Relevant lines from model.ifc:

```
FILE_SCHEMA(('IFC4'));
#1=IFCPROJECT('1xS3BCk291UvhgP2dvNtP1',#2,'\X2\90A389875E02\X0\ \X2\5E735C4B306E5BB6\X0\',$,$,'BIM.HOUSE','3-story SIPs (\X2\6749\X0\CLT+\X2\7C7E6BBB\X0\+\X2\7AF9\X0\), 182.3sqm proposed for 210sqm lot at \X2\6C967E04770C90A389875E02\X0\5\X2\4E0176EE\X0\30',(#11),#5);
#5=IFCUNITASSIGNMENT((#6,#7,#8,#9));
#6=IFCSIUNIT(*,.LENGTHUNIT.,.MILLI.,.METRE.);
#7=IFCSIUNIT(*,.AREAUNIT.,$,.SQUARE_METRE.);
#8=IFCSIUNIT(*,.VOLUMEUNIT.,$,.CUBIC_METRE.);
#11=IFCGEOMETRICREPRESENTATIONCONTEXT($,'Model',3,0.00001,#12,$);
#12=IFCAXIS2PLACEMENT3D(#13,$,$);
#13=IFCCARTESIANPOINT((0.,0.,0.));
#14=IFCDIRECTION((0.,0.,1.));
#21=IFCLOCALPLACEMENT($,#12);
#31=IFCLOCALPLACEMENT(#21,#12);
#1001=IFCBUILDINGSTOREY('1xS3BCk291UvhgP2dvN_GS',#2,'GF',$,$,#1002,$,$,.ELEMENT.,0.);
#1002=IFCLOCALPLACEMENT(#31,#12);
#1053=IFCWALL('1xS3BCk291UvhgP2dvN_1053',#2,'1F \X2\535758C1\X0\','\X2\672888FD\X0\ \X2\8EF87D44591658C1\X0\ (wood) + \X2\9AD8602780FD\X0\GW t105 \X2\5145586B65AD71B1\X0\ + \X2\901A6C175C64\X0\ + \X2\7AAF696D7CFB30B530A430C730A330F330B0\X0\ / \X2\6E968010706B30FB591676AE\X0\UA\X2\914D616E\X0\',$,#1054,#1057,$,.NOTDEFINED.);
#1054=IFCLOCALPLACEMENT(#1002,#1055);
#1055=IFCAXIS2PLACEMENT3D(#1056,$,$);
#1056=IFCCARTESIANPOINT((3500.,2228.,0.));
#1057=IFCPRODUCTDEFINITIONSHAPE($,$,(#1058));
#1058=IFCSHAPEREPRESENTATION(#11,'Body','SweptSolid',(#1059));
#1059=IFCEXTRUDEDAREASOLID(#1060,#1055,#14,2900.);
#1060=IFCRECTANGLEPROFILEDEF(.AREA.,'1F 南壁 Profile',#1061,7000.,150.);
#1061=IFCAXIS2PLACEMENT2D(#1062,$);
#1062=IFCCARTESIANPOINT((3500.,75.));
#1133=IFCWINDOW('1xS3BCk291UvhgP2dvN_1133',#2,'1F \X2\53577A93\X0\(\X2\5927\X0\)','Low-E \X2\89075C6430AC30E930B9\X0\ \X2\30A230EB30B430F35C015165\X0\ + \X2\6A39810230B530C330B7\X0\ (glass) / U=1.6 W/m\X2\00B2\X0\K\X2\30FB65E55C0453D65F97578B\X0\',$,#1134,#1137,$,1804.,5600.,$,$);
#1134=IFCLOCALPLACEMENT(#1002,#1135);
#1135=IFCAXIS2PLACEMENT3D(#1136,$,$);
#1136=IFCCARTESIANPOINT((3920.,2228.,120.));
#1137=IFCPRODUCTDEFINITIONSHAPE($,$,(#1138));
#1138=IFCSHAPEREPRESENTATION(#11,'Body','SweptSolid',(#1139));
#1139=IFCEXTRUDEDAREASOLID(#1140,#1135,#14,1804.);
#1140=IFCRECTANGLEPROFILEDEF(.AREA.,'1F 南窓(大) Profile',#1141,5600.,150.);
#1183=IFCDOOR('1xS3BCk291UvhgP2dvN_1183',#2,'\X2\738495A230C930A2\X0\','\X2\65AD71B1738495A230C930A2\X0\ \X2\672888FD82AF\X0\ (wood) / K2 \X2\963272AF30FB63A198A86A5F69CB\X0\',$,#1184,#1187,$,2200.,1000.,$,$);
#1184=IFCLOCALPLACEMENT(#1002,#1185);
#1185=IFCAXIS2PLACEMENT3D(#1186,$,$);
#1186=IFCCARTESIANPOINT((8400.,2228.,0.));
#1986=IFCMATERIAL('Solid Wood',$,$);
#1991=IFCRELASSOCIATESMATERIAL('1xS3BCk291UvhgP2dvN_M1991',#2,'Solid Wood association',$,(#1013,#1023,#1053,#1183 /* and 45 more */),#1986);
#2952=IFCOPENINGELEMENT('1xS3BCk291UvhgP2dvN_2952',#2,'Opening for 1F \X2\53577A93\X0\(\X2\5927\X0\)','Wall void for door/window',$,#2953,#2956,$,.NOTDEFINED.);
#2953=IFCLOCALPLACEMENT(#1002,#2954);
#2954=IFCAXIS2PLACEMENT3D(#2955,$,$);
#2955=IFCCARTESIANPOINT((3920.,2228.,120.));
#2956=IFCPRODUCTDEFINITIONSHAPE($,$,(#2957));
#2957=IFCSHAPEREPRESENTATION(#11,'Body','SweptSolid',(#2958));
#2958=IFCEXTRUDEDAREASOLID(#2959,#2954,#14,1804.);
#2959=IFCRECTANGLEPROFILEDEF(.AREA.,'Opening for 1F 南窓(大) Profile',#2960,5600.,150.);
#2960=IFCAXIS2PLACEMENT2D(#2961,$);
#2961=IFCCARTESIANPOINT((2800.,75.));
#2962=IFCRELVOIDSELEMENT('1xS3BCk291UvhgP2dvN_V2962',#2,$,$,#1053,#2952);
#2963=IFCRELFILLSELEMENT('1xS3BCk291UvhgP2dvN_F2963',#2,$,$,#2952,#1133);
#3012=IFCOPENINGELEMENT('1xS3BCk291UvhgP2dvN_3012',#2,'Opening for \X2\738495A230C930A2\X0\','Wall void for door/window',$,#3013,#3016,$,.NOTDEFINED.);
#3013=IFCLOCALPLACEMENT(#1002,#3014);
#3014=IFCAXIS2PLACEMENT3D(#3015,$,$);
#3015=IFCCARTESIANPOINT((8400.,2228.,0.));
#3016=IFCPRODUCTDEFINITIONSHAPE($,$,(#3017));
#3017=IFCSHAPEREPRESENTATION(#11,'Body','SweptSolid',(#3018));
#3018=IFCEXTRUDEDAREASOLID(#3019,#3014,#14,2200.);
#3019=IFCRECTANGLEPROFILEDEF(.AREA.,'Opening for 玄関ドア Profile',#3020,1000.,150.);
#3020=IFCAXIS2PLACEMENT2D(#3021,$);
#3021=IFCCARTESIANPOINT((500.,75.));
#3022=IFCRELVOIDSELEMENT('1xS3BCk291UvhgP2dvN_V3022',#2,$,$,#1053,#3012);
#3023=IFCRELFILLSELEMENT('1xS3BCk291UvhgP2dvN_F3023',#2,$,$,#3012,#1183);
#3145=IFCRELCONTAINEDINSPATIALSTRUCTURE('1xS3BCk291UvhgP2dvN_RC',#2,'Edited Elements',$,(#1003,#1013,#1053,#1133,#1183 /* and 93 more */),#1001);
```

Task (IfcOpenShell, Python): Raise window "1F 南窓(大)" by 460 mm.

```python
import numpy as np
import ifcopenshell
import ifcopenshell.api.geometry
import ifcopenshell.util.placement
import ifcopenshell.util.unit

model = ifcopenshell.open("model.ifc")
unit_scale = ifcopenshell.util.unit.calculate_unit_scale(model)

window = model.by_guid("1xS3BCk291UvhgP2dvN_1133")
opening = window.FillsVoids[0].RelatingOpeningElement
dz = 460.0

shift = np.array([0.0, 0.0, dz])
# The window is not placed relative to its opening, so move both.
for product in (opening, window):
    matrix = ifcopenshell.util.placement.get_local_placement(product.ObjectPlacement)
    matrix[:3, 3] += shift
    ifcopenshell.api.geometry.edit_object_placement(model, product=product, matrix=matrix, is_si=False)

print(f"moved by {dz * unit_scale:+.3f} m")

model.write("model-out.ifc")
```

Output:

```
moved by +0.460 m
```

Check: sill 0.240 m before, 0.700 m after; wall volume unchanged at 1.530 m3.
